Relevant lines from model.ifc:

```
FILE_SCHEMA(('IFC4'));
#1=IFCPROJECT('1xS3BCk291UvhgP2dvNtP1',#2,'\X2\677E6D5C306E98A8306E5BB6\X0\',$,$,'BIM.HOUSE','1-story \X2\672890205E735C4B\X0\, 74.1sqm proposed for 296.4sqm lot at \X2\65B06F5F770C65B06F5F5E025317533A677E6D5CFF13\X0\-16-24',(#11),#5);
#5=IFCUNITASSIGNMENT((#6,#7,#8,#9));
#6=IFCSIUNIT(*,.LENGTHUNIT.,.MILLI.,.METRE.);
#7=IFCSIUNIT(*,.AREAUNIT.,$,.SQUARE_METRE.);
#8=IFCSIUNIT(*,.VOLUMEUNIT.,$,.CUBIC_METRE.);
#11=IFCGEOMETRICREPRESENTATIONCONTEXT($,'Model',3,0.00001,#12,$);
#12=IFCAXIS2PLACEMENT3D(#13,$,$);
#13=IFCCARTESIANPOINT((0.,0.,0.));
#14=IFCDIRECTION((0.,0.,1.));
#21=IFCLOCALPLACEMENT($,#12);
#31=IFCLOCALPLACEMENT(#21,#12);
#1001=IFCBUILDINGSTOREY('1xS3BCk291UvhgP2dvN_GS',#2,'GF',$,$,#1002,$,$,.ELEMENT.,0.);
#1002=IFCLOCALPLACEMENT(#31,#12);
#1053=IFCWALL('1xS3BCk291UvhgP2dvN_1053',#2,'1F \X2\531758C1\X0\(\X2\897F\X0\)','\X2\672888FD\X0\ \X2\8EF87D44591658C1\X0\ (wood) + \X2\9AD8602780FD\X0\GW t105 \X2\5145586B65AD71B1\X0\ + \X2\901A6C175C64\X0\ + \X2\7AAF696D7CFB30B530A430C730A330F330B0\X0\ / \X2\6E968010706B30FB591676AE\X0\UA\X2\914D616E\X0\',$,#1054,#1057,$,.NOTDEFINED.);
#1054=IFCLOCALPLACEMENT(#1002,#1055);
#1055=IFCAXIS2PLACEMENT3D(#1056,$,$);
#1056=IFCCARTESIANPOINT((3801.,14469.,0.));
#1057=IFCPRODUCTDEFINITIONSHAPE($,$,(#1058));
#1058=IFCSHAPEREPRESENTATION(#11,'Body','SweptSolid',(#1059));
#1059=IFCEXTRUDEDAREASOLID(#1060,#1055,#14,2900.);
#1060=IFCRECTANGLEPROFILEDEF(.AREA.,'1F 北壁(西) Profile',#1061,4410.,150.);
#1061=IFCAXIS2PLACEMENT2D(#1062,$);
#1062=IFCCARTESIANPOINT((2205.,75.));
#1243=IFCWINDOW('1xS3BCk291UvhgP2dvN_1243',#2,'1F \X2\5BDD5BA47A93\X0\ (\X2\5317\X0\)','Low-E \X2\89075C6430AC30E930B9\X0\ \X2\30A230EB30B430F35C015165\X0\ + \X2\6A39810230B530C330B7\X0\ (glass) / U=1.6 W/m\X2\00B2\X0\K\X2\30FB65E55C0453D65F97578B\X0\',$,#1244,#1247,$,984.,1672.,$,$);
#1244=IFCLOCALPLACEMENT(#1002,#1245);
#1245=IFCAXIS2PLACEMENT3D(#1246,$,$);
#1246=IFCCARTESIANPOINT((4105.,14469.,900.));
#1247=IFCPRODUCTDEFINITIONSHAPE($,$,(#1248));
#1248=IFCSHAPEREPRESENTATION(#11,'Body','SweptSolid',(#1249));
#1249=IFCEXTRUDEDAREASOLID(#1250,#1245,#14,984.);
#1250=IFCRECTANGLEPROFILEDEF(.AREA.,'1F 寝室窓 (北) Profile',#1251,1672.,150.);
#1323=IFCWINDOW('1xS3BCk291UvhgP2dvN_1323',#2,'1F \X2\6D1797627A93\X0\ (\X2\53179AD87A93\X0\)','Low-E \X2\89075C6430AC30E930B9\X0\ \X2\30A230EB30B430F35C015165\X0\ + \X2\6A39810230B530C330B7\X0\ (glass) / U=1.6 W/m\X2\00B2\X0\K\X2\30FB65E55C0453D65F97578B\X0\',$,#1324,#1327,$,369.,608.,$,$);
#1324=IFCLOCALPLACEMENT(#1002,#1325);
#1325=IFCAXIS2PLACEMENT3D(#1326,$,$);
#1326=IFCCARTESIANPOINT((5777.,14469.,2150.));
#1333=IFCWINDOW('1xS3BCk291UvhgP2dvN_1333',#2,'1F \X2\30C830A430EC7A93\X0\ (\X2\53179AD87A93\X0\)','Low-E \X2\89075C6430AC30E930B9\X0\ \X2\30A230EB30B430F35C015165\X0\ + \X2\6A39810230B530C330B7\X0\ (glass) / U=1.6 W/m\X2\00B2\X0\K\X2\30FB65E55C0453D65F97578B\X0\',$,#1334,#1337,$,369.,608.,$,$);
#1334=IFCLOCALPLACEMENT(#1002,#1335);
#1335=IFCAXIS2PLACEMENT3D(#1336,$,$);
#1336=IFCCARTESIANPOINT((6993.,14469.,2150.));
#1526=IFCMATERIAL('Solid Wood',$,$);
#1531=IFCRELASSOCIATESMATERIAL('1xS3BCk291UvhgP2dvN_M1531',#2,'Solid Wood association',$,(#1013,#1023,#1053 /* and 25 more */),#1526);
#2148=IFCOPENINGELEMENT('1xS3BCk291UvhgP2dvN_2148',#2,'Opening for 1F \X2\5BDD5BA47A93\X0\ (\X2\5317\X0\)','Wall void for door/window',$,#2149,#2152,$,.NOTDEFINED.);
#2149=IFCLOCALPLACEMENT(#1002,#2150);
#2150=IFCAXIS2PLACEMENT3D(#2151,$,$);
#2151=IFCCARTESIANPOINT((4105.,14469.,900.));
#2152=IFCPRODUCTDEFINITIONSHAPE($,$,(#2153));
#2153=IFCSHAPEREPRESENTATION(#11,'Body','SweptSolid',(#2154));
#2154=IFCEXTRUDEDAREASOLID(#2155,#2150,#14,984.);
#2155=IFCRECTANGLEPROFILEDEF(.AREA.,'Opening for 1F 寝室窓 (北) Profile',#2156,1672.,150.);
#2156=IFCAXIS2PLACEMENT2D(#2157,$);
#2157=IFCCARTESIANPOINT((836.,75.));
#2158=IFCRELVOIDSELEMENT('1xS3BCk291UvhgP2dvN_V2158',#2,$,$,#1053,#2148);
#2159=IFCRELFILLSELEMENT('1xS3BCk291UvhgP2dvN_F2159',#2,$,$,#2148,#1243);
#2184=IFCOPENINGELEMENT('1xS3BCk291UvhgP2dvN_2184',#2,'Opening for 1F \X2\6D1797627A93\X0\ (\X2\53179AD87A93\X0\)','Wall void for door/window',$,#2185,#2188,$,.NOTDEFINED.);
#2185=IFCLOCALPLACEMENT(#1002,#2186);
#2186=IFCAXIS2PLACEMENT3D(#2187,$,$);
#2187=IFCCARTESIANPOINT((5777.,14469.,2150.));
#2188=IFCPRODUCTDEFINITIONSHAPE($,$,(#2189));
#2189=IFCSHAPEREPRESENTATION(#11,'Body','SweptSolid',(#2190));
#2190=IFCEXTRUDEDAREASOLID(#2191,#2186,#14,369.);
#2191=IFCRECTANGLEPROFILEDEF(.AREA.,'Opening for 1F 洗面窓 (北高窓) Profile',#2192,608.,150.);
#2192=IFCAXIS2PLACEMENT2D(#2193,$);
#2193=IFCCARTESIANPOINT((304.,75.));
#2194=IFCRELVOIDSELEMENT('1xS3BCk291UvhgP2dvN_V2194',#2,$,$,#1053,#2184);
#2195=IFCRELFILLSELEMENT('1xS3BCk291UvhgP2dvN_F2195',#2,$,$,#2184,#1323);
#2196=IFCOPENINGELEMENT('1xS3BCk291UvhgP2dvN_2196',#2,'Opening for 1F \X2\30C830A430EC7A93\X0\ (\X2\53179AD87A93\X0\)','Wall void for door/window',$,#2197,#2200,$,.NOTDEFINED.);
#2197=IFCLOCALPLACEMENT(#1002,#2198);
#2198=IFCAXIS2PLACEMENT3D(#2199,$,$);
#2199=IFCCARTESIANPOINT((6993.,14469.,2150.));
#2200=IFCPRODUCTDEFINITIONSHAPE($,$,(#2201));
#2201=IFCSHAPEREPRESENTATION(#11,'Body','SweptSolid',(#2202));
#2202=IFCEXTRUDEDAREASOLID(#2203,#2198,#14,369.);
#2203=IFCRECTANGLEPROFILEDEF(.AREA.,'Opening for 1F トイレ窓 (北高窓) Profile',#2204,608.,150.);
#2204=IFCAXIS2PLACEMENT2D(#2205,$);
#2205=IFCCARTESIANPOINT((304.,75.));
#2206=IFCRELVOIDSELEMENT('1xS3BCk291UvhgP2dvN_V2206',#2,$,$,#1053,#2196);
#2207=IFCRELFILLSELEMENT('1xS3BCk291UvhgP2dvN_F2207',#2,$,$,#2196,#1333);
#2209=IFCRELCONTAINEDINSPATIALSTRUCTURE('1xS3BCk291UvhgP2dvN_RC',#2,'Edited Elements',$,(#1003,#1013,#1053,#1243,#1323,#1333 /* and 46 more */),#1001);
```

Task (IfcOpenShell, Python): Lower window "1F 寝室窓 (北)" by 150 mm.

```python
import numpy as np
import ifcopenshell
import ifcopenshell.api.geometry
import ifcopenshell.util.placement
import ifcopenshell.util.unit

model = ifcopenshell.open("model.ifc")
unit_scale = ifcopenshell.util.unit.calculate_unit_scale(model)

window = model.by_guid("1xS3BCk291UvhgP2dvN_1243")
opening = window.FillsVoids[0].RelatingOpeningElement
dz = -0.15 / unit_scale

shift = np.array([0.0, 0.0, dz])
# The window is not placed relative to its opening, so move both.
for product in (opening, window):
    matrix = ifcopenshell.util.placement.get_local_placement(product.ObjectPlacement)
    matrix[:3, 3] += shift
    ifcopenshell.api.geometry.edit_object_placement(model, product=product, matrix=matrix, is_si=False)

print(f"moved by {dz * unit_scale:+.3f} m")

model.write("model-out.ifc")
```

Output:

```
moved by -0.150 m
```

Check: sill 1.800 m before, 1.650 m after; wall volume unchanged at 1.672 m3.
